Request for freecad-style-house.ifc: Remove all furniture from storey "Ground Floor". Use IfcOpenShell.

First a look at what the model holds.

```python
import ifcopenshell
import ifcopenshell.util.element

model = ifcopenshell.open("freecad-style-house.ifc")
print(model.schema)
storey = next(s for s in model.by_type("IfcBuildingStorey") if s.Name == "Ground Floor")
furniture = [e for e in ifcopenshell.util.element.get_decomposition(storey) if e.is_a("IfcFurnishingElement")]
seen = {}
for e in furniture:
    element_type = ifcopenshell.util.element.get_type(e)
    name = element_type.Name if element_type not in (None, e) else None
    seen[name] = seen.get(name, 0) + 1
for name, count in sorted(seen.items(), key=str):
    print(count, "x", name)
```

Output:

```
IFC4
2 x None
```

```python
import ifcopenshell
import ifcopenshell.api.root
import ifcopenshell.util.element

model = ifcopenshell.open("freecad-style-house.ifc")

storey = next(s for s in model.by_type("IfcBuildingStorey") if s.Name == "Ground Floor")
furniture = [e for e in ifcopenshell.util.element.get_decomposition(storey) if e.is_a("IfcFurnishingElement")]

for e in furniture:
    ifcopenshell.api.root.remove_product(model, product=e)
print(len(furniture), "removed")

model.write("freecad-style-house_edited.ifc")
```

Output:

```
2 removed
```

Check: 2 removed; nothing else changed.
